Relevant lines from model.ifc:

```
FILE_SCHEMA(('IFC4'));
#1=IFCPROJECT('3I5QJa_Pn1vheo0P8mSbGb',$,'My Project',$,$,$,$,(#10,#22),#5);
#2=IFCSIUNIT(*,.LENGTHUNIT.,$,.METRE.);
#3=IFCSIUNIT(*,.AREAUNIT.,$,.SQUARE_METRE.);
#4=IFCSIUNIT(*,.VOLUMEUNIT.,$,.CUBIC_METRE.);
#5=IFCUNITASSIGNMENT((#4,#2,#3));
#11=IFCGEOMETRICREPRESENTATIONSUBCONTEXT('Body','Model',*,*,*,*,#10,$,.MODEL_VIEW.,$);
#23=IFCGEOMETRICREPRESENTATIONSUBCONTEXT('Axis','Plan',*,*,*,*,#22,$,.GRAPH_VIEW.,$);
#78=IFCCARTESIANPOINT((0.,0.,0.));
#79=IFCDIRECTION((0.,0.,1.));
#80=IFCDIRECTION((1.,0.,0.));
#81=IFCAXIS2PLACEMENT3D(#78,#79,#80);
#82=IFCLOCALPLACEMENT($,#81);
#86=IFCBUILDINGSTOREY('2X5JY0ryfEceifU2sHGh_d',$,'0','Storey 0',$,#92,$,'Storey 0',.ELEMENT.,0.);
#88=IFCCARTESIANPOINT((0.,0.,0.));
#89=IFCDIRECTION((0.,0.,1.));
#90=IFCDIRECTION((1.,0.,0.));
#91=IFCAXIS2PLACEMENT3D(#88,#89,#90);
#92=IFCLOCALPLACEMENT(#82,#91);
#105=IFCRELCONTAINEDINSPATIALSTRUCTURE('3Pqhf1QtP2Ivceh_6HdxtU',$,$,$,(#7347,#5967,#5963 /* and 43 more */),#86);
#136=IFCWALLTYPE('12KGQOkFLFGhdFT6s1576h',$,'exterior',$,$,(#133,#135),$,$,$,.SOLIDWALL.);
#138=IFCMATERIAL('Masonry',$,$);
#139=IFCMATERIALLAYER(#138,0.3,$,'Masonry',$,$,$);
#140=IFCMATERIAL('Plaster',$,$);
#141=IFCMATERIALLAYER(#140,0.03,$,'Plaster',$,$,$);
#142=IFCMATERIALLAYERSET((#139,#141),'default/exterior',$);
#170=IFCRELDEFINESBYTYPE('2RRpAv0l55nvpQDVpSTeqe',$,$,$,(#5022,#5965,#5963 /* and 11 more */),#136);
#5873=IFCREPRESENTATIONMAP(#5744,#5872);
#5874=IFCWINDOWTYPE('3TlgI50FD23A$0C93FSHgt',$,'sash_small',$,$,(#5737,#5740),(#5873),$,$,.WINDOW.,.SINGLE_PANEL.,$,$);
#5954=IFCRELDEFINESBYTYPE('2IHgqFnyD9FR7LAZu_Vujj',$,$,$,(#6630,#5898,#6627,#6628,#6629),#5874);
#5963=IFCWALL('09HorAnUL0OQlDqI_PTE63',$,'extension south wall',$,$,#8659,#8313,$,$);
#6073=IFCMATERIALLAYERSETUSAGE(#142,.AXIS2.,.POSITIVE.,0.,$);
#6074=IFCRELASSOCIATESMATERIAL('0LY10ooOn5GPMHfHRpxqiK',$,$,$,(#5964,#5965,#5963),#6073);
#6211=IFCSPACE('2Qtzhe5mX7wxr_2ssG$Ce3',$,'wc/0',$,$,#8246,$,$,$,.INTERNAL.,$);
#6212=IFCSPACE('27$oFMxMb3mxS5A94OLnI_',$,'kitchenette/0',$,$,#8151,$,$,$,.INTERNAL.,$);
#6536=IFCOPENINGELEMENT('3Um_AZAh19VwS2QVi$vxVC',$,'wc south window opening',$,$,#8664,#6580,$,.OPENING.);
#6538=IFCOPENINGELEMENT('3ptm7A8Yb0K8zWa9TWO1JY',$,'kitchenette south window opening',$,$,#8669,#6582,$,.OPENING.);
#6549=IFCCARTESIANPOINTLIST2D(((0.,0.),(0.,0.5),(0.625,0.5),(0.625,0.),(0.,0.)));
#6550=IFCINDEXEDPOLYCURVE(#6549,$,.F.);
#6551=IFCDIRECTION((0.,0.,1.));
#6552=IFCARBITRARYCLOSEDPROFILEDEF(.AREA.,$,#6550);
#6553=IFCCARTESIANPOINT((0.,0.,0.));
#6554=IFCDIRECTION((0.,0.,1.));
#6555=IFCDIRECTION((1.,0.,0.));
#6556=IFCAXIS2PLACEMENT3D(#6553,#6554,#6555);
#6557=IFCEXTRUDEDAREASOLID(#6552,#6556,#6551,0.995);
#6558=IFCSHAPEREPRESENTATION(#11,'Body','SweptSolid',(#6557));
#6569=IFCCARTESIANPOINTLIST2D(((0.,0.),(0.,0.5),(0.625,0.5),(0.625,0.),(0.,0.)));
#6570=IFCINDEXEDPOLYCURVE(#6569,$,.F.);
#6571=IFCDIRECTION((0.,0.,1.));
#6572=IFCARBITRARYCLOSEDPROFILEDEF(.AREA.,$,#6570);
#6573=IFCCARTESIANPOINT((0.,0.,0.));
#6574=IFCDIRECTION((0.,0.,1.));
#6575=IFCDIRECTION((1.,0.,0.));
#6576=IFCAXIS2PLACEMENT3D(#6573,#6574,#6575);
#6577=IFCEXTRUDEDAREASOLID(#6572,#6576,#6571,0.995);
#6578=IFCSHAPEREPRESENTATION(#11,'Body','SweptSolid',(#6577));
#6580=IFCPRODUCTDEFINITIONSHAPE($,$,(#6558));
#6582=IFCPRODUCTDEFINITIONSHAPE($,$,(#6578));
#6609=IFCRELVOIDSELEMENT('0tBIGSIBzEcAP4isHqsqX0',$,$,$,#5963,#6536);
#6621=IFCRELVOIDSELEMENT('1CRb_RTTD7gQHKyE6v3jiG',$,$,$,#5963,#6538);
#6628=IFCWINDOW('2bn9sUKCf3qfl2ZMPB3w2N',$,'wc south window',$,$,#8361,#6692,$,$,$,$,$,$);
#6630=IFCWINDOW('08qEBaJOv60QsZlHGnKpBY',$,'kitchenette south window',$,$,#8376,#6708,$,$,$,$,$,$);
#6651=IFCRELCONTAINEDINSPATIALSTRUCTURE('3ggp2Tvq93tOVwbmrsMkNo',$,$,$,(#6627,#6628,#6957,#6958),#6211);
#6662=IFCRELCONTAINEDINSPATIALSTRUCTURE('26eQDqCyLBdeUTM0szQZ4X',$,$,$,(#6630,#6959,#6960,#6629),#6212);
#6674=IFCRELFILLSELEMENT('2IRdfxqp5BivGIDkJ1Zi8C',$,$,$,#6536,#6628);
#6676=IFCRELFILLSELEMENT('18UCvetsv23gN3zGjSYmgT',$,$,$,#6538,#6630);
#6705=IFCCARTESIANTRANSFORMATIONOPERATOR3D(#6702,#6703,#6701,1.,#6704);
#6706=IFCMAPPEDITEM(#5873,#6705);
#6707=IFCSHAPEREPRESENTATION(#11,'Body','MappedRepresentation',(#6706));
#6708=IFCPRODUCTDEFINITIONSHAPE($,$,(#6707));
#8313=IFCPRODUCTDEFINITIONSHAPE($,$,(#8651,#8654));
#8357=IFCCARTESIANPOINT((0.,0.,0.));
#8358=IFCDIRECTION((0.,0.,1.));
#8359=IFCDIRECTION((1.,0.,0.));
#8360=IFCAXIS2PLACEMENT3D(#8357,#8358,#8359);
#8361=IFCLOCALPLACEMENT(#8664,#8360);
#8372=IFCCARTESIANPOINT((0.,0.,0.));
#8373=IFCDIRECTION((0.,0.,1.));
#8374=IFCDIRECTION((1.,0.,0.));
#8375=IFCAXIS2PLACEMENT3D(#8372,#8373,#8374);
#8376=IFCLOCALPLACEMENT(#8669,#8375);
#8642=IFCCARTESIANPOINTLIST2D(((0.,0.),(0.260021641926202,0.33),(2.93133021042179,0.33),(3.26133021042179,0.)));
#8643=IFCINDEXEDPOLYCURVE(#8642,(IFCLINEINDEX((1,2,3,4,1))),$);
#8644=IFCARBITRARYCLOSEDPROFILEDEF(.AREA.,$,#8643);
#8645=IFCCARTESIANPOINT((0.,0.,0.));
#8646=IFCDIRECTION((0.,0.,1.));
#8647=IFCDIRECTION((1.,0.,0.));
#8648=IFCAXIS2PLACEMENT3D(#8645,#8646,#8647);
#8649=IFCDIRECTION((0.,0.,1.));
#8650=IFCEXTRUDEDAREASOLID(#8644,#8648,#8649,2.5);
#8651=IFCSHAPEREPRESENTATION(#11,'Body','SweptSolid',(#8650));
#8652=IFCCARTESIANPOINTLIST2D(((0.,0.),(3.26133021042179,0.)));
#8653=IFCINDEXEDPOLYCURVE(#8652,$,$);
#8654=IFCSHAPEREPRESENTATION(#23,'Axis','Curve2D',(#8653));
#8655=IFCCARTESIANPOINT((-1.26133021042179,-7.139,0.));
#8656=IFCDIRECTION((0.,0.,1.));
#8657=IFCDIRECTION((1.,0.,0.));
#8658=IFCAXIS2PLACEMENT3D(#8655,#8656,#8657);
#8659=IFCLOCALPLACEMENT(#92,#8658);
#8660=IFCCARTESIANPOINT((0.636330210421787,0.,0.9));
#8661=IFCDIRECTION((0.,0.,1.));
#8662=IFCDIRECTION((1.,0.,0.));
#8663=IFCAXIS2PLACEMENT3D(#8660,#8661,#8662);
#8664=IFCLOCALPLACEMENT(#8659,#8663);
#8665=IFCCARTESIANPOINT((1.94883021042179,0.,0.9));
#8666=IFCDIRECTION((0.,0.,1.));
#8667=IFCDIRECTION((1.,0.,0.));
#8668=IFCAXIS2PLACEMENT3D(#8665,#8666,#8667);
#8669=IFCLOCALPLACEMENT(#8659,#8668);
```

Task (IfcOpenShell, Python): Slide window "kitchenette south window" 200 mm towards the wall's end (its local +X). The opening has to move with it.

```python
import ifcopenshell
import ifcopenshell.api.geometry
import ifcopenshell.util.placement
import ifcopenshell.util.unit

model = ifcopenshell.open("model.ifc")
unit_scale = ifcopenshell.util.unit.calculate_unit_scale(model)

window = model.by_id(6630)
opening = window.FillsVoids[0].RelatingOpeningElement
wall = opening.VoidsElements[0].RelatingBuildingElement

wall_matrix = ifcopenshell.util.placement.get_local_placement(wall.ObjectPlacement)
shift = wall_matrix[:3, 0] * 0.2 / unit_scale
before = ifcopenshell.util.placement.get_local_placement(window.ObjectPlacement)[:3, 3].copy()

# The window is placed relative to its opening, so it follows when the opening moves.
matrix = ifcopenshell.util.placement.get_local_placement(opening.ObjectPlacement)
matrix[:3, 3] += shift
ifcopenshell.api.geometry.edit_object_placement(
    model, product=opening, matrix=matrix, is_si=False, should_transform_children=True
)

after = ifcopenshell.util.placement.get_local_placement(window.ObjectPlacement)[:3, 3]
print("window moved by", (after - before).round(3) + 0.0)

model.write("model_edited.ifc")
```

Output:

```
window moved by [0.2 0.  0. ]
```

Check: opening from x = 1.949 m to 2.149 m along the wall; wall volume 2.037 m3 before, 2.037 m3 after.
